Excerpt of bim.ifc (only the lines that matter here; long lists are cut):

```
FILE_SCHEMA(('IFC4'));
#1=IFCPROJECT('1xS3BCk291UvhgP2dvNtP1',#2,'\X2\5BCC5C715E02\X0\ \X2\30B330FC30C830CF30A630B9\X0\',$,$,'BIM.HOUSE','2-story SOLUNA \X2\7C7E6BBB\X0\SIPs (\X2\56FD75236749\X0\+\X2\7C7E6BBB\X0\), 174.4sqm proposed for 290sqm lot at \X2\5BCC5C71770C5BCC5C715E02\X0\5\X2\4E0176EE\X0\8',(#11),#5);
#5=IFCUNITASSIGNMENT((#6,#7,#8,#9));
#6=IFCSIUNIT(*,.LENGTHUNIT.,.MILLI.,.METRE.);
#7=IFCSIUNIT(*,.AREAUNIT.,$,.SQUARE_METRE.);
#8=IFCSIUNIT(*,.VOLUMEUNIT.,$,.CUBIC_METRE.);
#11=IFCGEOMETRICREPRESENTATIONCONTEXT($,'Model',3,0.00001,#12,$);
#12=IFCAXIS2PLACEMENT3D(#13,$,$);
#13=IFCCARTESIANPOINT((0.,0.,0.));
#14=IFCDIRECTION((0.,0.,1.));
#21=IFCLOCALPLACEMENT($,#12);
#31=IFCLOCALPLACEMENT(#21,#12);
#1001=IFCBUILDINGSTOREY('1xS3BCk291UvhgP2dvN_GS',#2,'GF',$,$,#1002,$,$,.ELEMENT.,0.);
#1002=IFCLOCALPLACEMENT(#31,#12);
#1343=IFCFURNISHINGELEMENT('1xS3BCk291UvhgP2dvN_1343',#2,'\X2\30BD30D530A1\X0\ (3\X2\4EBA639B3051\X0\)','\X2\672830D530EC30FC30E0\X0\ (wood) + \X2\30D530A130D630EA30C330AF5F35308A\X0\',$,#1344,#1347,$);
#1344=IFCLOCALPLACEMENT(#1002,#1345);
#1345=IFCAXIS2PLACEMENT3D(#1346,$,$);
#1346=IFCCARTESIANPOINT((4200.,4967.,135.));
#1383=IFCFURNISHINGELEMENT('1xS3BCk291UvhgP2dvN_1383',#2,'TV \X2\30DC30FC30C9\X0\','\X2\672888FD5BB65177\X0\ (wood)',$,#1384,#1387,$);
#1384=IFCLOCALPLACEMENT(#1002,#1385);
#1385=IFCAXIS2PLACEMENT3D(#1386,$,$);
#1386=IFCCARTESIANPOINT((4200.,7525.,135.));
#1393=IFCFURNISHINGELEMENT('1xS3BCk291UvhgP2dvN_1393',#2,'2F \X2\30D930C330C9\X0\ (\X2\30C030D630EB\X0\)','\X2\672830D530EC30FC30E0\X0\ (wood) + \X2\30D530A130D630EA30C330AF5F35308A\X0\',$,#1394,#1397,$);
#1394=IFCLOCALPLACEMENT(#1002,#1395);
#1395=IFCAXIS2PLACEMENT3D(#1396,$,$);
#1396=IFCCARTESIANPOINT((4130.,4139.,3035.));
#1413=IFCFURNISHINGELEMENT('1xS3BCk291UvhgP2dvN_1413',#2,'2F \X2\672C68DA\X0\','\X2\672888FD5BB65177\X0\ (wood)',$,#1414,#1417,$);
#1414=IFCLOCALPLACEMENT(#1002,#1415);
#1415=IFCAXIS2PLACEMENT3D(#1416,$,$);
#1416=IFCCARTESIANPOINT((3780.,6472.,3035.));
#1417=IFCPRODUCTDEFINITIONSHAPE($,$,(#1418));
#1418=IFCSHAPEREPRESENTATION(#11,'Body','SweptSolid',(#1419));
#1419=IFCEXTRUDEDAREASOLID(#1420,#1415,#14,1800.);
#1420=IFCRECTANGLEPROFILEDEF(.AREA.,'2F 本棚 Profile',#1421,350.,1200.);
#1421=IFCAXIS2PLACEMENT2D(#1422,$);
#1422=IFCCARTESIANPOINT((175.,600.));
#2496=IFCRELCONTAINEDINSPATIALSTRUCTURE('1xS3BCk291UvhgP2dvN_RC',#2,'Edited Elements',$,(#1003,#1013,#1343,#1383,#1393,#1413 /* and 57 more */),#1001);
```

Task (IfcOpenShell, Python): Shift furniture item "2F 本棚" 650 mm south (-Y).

```python
import ifcopenshell
import ifcopenshell.api.geometry
import ifcopenshell.util.placement
import ifcopenshell.util.unit

model = ifcopenshell.open("bim.ifc")
unit_scale = ifcopenshell.util.unit.calculate_unit_scale(model)

item = model.by_id(1413)
matrix = ifcopenshell.util.placement.get_local_placement(item.ObjectPlacement)
matrix[1, 3] -= 0.65 / unit_scale
ifcopenshell.api.geometry.edit_object_placement(model, product=item, matrix=matrix, is_si=False)

print(ifcopenshell.util.placement.get_local_placement(item.ObjectPlacement).round(3) + 0.0)

model.write("bim-out.ifc")
```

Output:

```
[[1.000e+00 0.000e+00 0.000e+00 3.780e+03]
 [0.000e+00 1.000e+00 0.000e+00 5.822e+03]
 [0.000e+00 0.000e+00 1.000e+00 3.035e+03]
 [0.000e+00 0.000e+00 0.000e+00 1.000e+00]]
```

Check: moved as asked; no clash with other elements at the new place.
